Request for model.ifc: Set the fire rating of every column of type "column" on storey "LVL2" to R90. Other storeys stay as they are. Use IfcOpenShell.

First a look at what the model holds.

```python
import ifcopenshell
import ifcopenshell.util.element

model = ifcopenshell.open("model.ifc")
print(model.schema)
storey = next(s for s in model.by_type("IfcBuildingStorey") if s.Name == "LVL2")
columns = [e for e in ifcopenshell.util.element.get_decomposition(storey) if e.is_a("IfcColumn")]
seen = {}
for e in columns:
    element_type = ifcopenshell.util.element.get_type(e)
    key = (element_type.Name if element_type != e and element_type else None, ifcopenshell.util.element.get_pset(e, "Pset_ColumnCommon", "FireRating"))
    seen[key] = seen.get(key, 0) + 1
for (name, value), count in sorted(seen.items(), key=str):
    print(count, "x", name, "|", value)
```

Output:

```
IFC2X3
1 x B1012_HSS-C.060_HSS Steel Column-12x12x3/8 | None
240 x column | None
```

```python
import ifcopenshell
import ifcopenshell.api.pset
import ifcopenshell.util.element

model = ifcopenshell.open("model.ifc")

storey = next(s for s in model.by_type("IfcBuildingStorey") if s.Name == "LVL2")
columns = [e for e in ifcopenshell.util.element.get_decomposition(storey) if e.is_a("IfcColumn")]

count = 0
for e in columns:
    element_type = ifcopenshell.util.element.get_type(e)
    if element_type in (None, e) or element_type.Name != "column":
        continue
    # add_pset returns the element's existing set when there is one.
    pset = ifcopenshell.api.pset.add_pset(model, product=e, name="Pset_ColumnCommon")
    ifcopenshell.api.pset.edit_pset(model, pset=pset, properties={"FireRating": "R90"})
    count += 1

print(count, "columns updated")

model.write("model_rev.ifc")
```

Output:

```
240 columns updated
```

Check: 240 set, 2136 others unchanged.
